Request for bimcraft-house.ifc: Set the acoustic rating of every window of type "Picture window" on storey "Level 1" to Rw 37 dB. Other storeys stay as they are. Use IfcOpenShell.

First a look at what the model holds.

```python
import ifcopenshell
import ifcopenshell.util.element

model = ifcopenshell.open("bimcraft-house.ifc")
print(model.schema)
storey = next(s for s in model.by_type("IfcBuildingStorey") if s.Name == "Level 1")
windows = [e for e in ifcopenshell.util.element.get_decomposition(storey) if e.is_a("IfcWindow")]
seen = {}
for e in windows:
    element_type = ifcopenshell.util.element.get_type(e)
    key = (element_type.Name if element_type != e and element_type else None, ifcopenshell.util.element.get_pset(e, "Pset_WindowCommon", "AcousticRating"))
    seen[key] = seen.get(key, 0) + 1
for (name, value), count in sorted(seen.items(), key=str):
    print(count, "x", name, "|", value)
```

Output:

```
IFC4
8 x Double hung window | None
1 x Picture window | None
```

```python
import ifcopenshell
import ifcopenshell.api.pset
import ifcopenshell.util.element

model = ifcopenshell.open("bimcraft-house.ifc")

storey = next(s for s in model.by_type("IfcBuildingStorey") if s.Name == "Level 1")
windows = [e for e in ifcopenshell.util.element.get_decomposition(storey) if e.is_a("IfcWindow")]

count = 0
for e in windows:
    element_type = ifcopenshell.util.element.get_type(e)
    if element_type in (None, e) or element_type.Name != "Picture window":
        continue
    # add_pset returns the element's existing set when there is one.
    pset = ifcopenshell.api.pset.add_pset(model, product=e, name="Pset_WindowCommon")
    ifcopenshell.api.pset.edit_pset(model, pset=pset, properties={"AcousticRating": "Rw 37 dB"})
    count += 1

print(count, "windows updated")

model.write("bimcraft-house_rev.ifc")
```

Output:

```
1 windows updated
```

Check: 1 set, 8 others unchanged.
